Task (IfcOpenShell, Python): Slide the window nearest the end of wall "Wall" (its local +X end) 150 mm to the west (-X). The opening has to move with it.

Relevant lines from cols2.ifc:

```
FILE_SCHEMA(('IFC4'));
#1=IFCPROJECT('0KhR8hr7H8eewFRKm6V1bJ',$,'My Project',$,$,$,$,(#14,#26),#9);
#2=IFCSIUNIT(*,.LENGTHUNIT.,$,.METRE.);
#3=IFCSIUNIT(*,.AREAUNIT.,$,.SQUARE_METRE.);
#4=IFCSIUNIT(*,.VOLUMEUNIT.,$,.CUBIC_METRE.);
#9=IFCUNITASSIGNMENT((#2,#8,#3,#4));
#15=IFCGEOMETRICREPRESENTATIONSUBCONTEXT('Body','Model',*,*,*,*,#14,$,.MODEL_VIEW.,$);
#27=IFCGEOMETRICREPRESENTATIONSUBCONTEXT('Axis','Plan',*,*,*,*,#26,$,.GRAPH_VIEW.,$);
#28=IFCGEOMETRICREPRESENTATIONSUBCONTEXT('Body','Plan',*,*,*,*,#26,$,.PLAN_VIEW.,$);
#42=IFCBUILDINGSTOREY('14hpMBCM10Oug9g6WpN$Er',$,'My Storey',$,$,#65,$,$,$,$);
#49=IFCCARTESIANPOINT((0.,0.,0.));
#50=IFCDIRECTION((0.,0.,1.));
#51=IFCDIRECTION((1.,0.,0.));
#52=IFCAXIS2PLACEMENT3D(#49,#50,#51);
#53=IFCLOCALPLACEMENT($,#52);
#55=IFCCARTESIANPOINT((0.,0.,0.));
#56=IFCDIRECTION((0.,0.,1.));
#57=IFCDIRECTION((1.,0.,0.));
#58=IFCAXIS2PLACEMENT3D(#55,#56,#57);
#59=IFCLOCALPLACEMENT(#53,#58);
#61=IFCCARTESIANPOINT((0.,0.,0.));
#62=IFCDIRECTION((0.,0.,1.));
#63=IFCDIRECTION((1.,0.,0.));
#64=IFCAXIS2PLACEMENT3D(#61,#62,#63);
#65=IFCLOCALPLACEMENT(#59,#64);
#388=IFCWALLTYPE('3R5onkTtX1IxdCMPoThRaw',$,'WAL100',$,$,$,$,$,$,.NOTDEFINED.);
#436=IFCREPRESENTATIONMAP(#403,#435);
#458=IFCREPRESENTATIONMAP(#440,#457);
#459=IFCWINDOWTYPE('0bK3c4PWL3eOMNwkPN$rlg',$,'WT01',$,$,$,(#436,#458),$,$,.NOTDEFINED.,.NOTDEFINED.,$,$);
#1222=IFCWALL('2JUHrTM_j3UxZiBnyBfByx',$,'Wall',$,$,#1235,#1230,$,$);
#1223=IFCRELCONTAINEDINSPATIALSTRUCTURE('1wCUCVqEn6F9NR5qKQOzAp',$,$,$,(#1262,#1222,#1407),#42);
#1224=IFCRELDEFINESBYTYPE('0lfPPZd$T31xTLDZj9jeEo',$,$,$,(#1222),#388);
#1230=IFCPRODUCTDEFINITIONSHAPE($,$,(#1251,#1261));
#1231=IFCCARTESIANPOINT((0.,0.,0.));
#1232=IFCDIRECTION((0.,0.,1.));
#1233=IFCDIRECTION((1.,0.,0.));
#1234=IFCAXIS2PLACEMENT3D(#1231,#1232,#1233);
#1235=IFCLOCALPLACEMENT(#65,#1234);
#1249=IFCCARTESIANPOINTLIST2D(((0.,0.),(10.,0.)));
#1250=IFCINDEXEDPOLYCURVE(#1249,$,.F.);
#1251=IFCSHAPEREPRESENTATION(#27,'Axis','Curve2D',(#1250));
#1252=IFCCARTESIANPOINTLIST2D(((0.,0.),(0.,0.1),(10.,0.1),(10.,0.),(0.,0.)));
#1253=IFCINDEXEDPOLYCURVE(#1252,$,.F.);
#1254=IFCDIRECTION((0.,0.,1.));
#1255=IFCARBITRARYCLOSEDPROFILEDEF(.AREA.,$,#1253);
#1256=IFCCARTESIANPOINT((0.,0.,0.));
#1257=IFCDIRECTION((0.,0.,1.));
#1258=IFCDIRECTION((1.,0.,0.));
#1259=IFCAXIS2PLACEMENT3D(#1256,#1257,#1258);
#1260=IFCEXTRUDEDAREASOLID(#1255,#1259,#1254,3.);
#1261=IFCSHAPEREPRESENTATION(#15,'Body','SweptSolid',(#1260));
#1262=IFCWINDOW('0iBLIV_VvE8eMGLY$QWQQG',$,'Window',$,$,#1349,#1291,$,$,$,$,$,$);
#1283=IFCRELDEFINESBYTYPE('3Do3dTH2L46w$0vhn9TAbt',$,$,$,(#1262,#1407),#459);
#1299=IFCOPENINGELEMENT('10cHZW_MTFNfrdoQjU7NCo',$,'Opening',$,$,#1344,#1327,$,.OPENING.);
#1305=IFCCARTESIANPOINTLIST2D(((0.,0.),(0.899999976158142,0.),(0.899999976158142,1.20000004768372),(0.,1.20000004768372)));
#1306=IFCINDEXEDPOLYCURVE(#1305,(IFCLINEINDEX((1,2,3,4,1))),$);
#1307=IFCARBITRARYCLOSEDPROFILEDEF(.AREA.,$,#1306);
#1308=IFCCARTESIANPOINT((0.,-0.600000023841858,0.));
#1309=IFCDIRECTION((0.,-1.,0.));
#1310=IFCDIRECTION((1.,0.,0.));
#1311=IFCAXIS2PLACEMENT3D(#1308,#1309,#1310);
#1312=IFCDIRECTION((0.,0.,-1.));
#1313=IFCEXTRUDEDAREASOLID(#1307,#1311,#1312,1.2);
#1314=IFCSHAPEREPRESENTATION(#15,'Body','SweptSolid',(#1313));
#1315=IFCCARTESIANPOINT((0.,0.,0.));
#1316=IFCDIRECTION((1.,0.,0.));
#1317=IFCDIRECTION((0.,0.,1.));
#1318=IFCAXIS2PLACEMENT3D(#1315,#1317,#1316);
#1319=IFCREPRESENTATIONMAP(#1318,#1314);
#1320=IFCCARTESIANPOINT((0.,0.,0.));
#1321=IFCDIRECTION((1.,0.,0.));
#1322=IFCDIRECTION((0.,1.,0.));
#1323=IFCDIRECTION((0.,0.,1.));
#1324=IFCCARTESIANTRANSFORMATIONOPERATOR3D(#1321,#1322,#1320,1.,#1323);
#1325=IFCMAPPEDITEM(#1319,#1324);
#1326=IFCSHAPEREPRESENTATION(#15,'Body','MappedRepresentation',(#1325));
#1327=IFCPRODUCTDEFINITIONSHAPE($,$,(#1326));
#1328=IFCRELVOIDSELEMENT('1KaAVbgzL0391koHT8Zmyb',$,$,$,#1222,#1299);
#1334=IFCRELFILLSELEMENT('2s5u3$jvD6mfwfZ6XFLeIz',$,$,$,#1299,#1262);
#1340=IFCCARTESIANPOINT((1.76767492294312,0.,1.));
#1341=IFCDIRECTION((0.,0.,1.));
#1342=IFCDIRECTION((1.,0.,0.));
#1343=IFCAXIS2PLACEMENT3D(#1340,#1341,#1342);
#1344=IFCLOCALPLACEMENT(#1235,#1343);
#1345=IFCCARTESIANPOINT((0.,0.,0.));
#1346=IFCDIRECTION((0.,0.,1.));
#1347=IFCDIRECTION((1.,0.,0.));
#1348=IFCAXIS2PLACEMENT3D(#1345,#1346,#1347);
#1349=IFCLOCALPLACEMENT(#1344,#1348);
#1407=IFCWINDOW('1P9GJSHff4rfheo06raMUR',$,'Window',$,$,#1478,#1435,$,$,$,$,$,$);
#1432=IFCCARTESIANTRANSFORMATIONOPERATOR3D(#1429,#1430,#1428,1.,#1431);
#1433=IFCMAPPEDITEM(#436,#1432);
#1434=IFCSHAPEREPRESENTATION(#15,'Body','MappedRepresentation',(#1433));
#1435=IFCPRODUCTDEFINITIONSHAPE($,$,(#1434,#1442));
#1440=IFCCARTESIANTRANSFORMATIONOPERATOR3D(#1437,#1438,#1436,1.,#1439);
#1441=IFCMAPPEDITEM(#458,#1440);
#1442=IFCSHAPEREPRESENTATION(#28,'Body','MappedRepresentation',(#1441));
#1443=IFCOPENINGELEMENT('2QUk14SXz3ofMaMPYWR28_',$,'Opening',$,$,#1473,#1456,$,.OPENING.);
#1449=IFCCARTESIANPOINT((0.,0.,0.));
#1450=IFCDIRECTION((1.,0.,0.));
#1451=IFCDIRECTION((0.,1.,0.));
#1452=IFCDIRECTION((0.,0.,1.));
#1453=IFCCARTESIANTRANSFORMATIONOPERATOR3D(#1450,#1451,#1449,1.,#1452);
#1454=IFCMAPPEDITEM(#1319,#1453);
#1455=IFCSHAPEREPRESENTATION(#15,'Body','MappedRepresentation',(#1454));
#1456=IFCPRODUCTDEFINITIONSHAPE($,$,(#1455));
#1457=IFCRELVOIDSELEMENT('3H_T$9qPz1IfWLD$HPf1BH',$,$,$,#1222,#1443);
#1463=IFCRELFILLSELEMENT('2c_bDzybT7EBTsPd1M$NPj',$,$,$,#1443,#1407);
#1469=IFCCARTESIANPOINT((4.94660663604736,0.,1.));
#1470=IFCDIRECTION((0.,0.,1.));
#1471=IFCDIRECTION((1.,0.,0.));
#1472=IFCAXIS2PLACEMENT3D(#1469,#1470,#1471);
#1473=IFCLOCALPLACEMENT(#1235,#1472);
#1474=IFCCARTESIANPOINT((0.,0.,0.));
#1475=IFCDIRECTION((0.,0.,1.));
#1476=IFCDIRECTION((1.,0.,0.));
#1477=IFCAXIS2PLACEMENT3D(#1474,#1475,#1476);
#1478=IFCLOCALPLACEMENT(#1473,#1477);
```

```python
import ifcopenshell
import ifcopenshell.api.geometry
import ifcopenshell.util.placement
import ifcopenshell.util.unit

model = ifcopenshell.open("cols2.ifc")
unit_scale = ifcopenshell.util.unit.calculate_unit_scale(model)

window = model.by_guid("1P9GJSHff4rfheo06raMUR")
opening = window.FillsVoids[0].RelatingOpeningElement
wall = opening.VoidsElements[0].RelatingBuildingElement

wall_matrix = ifcopenshell.util.placement.get_local_placement(wall.ObjectPlacement)
shift = wall_matrix[:3, 0] * -0.15 / unit_scale
before = ifcopenshell.util.placement.get_local_placement(window.ObjectPlacement)[:3, 3].copy()

# The window is placed relative to its opening, so it follows when the opening moves.
matrix = ifcopenshell.util.placement.get_local_placement(opening.ObjectPlacement)
matrix[:3, 3] += shift
ifcopenshell.api.geometry.edit_object_placement(
    model, product=opening, matrix=matrix, is_si=False, should_transform_children=True
)

after = ifcopenshell.util.placement.get_local_placement(window.ObjectPlacement)[:3, 3]
print("window moved by", (after - before).round(3) + 0.0)

model.write("cols2-out.ifc")
```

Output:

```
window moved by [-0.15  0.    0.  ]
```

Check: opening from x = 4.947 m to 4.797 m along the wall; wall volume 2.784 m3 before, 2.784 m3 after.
